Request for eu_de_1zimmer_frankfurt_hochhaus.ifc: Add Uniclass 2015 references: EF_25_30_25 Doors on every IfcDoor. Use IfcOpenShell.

First a look at what the model holds.

```python
import ifcopenshell

model = ifcopenshell.open("eu_de_1zimmer_frankfurt_hochhaus.ifc")
print(model.schema)
print("classifications:", [c.Name for c in model.by_type("IfcClassification")])
for ifc_class in ("IfcDoor", "IfcRoof", "IfcStair", "IfcWall", "IfcWindow"):
    print(ifc_class, len(model.by_type(ifc_class)))
```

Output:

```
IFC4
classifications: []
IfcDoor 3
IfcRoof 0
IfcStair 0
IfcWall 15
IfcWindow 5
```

```python
import ifcopenshell
import ifcopenshell.api.classification

model = ifcopenshell.open("eu_de_1zimmer_frankfurt_hochhaus.ifc")

system = ifcopenshell.api.classification.add_classification(model, classification="Uniclass 2015")

codes = {
    "IfcDoor": ("EF_25_30_25", "Doors"),
}
for ifc_class, (code, name) in codes.items():
    products = model.by_type(ifc_class)
    ifcopenshell.api.classification.add_reference(
        model, products=products, classification=system, identification=code, name=name
    )
    print(code, len(products))

model.write("eu_de_1zimmer_frankfurt_hochhaus_rev.ifc")
```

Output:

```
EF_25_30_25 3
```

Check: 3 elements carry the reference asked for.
